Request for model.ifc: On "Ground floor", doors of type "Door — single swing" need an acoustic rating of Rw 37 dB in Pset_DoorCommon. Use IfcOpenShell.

First a look at what the model holds.

```python
import ifcopenshell
import ifcopenshell.util.element

model = ifcopenshell.open("model.ifc")
print(model.schema)
storey = next(s for s in model.by_type("IfcBuildingStorey") if s.Name == "Ground floor")
doors = [e for e in ifcopenshell.util.element.get_decomposition(storey) if e.is_a("IfcDoor")]
seen = {}
for e in doors:
    element_type = ifcopenshell.util.element.get_type(e)
    key = (element_type.Name if element_type != e and element_type else None, ifcopenshell.util.element.get_pset(e, "Pset_DoorCommon", "AcousticRating"))
    seen[key] = seen.get(key, 0) + 1
for (name, value), count in sorted(seen.items(), key=str):
    print(count, "x", name, "|", value)
```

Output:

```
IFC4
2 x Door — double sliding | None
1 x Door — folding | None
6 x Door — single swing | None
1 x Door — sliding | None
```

```python
import ifcopenshell
import ifcopenshell.api.pset
import ifcopenshell.util.element

model = ifcopenshell.open("model.ifc")

storey = next(s for s in model.by_type("IfcBuildingStorey") if s.Name == "Ground floor")
doors = [e for e in ifcopenshell.util.element.get_decomposition(storey) if e.is_a("IfcDoor")]

count = 0
for e in doors:
    element_type = ifcopenshell.util.element.get_type(e)
    if element_type in (None, e) or element_type.Name != "Door — single swing":
        continue
    # add_pset returns the element's existing set when there is one.
    pset = ifcopenshell.api.pset.add_pset(model, product=e, name="Pset_DoorCommon")
    ifcopenshell.api.pset.edit_pset(model, pset=pset, properties={"AcousticRating": "Rw 37 dB"})
    count += 1

print(count, "doors updated")

model.write("model_edited.ifc")
```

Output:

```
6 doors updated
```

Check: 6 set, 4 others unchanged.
